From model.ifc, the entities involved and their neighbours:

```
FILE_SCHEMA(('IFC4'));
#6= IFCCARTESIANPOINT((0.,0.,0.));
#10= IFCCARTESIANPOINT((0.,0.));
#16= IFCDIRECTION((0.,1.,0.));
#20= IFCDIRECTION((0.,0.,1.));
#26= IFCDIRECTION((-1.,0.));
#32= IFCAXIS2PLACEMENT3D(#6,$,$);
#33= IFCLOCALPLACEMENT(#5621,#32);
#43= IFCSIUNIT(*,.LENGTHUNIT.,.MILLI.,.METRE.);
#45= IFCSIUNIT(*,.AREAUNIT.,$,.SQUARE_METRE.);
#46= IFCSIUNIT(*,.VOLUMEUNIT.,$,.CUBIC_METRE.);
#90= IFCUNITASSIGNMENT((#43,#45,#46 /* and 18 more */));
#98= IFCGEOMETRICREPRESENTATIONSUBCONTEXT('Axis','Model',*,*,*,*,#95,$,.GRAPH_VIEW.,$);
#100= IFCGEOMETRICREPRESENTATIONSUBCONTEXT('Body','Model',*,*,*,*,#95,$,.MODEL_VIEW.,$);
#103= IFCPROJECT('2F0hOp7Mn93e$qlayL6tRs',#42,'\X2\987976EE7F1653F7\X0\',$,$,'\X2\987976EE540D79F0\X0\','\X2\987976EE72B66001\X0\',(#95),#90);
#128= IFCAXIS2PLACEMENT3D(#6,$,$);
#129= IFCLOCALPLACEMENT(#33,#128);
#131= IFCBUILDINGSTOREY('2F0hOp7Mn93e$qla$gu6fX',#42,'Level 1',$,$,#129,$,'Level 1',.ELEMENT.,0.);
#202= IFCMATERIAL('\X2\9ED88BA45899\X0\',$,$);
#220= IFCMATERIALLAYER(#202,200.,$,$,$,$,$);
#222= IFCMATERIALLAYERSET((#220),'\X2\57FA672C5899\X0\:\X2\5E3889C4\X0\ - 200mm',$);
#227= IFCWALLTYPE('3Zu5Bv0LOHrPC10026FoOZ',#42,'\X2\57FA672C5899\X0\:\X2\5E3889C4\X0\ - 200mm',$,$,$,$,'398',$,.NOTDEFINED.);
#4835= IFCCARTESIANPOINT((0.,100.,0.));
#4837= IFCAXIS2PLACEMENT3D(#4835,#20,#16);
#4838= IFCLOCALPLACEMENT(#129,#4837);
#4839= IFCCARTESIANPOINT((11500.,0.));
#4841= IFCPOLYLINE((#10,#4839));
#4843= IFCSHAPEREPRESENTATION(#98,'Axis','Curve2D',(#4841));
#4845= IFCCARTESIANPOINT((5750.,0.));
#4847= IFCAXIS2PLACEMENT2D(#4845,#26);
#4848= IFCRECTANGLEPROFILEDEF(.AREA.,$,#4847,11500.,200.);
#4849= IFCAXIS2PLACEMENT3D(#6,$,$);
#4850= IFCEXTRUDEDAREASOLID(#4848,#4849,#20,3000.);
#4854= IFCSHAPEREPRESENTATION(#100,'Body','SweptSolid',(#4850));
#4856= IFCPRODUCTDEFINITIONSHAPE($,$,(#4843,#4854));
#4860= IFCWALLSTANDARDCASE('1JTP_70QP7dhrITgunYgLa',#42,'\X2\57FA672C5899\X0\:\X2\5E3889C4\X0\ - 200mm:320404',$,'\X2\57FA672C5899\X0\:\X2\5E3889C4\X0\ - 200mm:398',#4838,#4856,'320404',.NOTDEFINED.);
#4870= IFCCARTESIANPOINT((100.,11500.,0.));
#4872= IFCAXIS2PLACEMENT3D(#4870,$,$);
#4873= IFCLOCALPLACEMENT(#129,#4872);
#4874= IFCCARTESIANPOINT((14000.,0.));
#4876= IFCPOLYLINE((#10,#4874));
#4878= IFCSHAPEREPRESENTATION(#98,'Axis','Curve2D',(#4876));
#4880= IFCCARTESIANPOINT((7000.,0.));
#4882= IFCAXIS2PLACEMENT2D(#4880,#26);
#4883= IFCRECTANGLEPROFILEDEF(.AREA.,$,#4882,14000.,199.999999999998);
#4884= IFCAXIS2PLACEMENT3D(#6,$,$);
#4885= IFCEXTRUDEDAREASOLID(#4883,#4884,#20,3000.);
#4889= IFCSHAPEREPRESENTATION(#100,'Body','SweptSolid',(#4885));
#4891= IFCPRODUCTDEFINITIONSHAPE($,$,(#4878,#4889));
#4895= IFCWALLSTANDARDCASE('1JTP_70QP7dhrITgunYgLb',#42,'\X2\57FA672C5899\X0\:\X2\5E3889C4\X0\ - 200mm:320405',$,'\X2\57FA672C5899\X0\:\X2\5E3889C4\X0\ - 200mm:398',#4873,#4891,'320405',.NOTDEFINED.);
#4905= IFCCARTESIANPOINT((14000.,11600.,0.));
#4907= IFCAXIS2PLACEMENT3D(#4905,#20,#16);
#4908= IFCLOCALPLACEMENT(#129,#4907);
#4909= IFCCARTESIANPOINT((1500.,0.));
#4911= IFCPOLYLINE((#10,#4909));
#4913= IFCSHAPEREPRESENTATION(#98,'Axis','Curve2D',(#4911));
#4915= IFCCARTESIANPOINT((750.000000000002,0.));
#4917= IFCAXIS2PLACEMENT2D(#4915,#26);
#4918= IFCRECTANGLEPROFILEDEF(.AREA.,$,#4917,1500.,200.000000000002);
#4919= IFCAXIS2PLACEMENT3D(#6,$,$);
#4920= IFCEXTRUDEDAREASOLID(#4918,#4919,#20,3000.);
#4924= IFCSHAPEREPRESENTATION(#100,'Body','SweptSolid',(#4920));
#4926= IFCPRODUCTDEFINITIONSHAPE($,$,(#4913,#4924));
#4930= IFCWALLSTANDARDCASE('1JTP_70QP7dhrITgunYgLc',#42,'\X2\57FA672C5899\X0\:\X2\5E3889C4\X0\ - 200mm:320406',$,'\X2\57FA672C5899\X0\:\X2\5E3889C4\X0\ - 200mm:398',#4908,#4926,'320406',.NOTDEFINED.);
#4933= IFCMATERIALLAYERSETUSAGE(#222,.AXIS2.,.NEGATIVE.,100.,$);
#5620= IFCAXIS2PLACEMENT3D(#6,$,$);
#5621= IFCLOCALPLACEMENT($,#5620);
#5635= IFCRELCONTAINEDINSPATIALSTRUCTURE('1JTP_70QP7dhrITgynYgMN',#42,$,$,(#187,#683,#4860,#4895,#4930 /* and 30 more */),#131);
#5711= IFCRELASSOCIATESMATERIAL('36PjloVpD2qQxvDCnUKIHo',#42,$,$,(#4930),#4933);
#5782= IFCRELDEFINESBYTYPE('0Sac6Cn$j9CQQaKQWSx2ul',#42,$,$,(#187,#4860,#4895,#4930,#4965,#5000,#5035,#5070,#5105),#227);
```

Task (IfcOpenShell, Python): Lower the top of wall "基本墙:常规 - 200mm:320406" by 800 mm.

```python
import ifcopenshell
import ifcopenshell.geom
import ifcopenshell.util.representation
import ifcopenshell.util.shape
import ifcopenshell.util.unit

model = ifcopenshell.open("model.ifc")
unit_scale = ifcopenshell.util.unit.calculate_unit_scale(model)
settings = ifcopenshell.geom.settings()


def volume(element):
    """Net volume in cubic metres, openings subtracted."""
    shape = ifcopenshell.geom.create_shape(settings, element)
    return ifcopenshell.util.shape.get_volume(shape.geometry)


wall = model.by_guid("1JTP_70QP7dhrITgunYgLc")
before = volume(wall)

body = ifcopenshell.util.representation.get_representation(wall, "Model", "Body")
solid = body.Items[0]
old_height = solid.Depth
solid.Depth -= 0.8 / unit_scale
after = volume(wall)

print(f"height {old_height:g} -> {solid.Depth:g}, volume {before:.3f} -> {after:.3f} m3")

model.write("model_edited.ifc")
```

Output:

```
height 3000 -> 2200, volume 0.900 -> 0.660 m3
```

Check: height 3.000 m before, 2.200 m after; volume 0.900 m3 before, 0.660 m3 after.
